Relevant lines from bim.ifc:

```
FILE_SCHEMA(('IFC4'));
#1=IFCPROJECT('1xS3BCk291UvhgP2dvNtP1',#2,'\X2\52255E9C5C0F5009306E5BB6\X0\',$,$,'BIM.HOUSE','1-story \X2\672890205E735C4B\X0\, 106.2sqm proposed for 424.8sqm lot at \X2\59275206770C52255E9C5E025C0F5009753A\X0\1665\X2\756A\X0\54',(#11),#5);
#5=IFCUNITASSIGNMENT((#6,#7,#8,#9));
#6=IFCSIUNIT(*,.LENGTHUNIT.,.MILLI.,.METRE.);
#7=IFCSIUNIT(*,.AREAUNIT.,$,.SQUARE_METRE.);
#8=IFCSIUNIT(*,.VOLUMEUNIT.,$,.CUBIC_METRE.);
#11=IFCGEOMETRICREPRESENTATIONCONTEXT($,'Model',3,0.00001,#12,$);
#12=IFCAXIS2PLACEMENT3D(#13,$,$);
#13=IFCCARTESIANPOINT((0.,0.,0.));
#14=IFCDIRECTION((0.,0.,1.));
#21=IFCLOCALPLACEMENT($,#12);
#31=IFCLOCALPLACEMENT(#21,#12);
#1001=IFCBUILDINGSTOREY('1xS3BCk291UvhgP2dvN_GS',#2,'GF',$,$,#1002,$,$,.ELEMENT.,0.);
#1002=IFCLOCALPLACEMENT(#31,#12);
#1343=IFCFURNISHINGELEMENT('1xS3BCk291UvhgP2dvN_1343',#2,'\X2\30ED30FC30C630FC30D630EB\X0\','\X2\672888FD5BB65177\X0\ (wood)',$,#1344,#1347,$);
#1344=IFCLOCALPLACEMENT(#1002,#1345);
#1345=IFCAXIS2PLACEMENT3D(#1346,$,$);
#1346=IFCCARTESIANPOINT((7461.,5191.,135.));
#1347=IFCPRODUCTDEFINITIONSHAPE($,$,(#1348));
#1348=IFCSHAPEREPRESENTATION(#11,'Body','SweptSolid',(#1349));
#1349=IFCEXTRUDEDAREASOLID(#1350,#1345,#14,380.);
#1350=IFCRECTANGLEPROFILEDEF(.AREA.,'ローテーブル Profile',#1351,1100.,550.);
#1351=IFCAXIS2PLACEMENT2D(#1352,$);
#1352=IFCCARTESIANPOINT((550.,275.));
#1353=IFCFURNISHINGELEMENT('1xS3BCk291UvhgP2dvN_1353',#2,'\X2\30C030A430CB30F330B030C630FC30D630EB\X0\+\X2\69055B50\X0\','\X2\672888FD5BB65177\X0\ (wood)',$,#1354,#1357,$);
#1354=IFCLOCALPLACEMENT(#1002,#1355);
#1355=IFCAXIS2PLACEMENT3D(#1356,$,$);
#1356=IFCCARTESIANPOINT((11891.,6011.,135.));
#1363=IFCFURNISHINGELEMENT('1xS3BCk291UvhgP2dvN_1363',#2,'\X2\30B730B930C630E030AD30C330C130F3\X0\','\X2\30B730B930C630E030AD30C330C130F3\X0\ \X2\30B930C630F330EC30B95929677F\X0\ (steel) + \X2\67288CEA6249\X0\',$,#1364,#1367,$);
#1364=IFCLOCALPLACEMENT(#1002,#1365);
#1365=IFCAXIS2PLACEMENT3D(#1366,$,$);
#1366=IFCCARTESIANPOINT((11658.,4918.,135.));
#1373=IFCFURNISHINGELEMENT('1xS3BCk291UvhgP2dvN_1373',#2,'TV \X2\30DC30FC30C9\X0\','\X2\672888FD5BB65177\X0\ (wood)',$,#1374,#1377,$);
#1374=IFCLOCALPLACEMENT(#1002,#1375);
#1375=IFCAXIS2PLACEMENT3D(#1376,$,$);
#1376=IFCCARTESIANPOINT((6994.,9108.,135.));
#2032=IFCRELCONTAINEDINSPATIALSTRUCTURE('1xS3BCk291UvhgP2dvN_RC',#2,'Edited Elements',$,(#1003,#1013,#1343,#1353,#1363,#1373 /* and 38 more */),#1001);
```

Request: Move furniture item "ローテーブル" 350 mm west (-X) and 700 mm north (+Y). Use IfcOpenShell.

```python
import ifcopenshell
import ifcopenshell.api.geometry
import ifcopenshell.util.placement
import ifcopenshell.util.unit

model = ifcopenshell.open("bim.ifc")
unit_scale = ifcopenshell.util.unit.calculate_unit_scale(model)

item = model.by_id(1343)
matrix = ifcopenshell.util.placement.get_local_placement(item.ObjectPlacement)
matrix[0, 3] -= 0.35 / unit_scale
matrix[1, 3] += 0.7 / unit_scale
ifcopenshell.api.geometry.edit_object_placement(model, product=item, matrix=matrix, is_si=False)

print(ifcopenshell.util.placement.get_local_placement(item.ObjectPlacement).round(3) + 0.0)

model.write("bim_v2.ifc")
```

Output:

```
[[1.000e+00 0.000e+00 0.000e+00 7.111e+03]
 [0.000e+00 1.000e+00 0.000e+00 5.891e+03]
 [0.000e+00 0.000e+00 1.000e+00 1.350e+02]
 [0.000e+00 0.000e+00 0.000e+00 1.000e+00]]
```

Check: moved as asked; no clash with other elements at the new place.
